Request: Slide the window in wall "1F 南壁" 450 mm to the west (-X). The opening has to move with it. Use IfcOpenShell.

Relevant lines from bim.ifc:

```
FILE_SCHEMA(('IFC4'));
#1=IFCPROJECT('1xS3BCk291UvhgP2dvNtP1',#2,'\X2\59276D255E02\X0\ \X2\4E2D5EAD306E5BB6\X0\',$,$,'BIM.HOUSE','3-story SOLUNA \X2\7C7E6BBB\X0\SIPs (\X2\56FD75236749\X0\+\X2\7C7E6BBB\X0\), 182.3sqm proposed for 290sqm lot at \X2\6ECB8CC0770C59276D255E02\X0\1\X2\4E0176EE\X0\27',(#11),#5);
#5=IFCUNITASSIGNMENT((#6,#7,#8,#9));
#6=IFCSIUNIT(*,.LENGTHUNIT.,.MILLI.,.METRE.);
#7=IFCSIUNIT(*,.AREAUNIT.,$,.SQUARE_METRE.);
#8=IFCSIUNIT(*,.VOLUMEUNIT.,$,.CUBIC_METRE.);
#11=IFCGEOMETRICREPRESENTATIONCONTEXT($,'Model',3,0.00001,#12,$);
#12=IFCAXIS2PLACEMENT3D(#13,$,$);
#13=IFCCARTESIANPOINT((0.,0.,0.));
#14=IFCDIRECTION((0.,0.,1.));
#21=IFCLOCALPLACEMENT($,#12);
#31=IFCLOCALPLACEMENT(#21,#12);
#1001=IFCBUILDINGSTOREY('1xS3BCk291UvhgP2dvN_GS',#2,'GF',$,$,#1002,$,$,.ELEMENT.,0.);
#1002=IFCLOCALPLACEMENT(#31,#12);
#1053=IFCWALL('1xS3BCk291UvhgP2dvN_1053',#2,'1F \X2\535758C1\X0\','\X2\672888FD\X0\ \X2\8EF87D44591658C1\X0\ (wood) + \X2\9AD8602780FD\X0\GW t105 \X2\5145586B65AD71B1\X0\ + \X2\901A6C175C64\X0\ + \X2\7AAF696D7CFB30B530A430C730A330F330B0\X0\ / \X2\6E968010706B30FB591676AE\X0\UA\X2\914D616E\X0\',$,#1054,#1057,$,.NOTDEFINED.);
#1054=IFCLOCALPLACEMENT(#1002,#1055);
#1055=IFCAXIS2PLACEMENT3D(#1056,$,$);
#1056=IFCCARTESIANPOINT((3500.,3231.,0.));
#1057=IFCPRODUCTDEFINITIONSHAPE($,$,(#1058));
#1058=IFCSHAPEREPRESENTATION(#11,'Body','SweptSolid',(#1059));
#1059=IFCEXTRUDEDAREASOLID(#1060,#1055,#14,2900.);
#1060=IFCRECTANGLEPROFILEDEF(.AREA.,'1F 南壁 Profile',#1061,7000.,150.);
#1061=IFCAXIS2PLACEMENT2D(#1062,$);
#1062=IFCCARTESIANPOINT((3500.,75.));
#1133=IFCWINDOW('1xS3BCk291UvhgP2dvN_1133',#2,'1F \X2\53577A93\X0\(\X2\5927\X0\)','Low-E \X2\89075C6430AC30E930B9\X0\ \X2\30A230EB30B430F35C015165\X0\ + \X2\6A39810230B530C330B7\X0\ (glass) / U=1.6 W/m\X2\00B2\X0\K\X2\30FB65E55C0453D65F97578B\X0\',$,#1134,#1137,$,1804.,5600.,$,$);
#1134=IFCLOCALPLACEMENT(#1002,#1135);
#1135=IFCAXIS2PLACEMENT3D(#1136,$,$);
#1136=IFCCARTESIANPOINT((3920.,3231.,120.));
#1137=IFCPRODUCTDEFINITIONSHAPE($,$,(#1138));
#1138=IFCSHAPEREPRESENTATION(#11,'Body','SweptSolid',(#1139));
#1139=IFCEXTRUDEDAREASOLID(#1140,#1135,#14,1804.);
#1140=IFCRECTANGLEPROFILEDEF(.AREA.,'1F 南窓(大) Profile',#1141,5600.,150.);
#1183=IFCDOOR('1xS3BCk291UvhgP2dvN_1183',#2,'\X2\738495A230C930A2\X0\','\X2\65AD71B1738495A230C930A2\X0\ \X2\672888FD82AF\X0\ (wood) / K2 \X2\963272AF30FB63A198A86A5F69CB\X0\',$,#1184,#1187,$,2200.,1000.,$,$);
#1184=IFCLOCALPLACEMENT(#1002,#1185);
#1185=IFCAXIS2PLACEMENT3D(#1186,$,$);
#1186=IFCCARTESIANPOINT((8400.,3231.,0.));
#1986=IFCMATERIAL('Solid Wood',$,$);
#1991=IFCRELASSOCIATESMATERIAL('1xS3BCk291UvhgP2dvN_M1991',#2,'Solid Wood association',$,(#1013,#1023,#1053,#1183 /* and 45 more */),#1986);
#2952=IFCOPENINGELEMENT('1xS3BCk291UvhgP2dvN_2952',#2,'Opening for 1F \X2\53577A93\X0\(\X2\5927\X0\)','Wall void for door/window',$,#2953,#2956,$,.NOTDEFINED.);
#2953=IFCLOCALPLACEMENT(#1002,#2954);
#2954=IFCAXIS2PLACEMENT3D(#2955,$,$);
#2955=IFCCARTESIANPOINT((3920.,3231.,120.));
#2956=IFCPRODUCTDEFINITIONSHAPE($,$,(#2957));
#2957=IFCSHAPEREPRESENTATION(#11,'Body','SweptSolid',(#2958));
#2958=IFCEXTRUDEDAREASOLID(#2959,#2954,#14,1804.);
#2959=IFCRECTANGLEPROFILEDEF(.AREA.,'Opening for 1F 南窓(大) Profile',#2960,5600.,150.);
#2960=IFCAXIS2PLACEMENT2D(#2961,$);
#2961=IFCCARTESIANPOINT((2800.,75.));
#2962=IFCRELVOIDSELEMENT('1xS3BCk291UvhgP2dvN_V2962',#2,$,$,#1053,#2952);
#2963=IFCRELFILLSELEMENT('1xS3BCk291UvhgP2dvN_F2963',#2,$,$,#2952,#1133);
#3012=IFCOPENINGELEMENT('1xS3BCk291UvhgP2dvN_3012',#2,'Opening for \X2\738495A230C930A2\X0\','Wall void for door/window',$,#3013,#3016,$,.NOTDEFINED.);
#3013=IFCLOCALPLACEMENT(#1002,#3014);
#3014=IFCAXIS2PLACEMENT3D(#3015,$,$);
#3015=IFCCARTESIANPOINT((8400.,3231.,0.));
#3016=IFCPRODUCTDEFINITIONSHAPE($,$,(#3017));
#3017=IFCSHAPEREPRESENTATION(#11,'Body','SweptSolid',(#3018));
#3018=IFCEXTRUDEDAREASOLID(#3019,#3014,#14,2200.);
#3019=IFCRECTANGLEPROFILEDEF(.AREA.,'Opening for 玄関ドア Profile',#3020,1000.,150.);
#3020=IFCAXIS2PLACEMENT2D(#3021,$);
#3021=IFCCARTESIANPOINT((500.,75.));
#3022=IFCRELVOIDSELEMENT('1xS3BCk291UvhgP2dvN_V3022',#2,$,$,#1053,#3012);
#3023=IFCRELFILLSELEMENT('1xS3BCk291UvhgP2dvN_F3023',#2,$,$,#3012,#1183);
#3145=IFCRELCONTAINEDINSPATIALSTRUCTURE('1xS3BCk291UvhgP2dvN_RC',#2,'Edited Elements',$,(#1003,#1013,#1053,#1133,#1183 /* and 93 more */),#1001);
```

```python
import ifcopenshell
import ifcopenshell.api.geometry
import ifcopenshell.util.placement

model = ifcopenshell.open("bim.ifc")

window = model.by_guid("1xS3BCk291UvhgP2dvN_1133")
opening = window.FillsVoids[0].RelatingOpeningElement
wall = opening.VoidsElements[0].RelatingBuildingElement

wall_matrix = ifcopenshell.util.placement.get_local_placement(wall.ObjectPlacement)
shift = wall_matrix[:3, 0] * -450.0
before = ifcopenshell.util.placement.get_local_placement(window.ObjectPlacement)[:3, 3].copy()

# The window is not placed relative to its opening, so move both.
for product in (opening, window):
    matrix = ifcopenshell.util.placement.get_local_placement(product.ObjectPlacement)
    matrix[:3, 3] += shift
    ifcopenshell.api.geometry.edit_object_placement(model, product=product, matrix=matrix, is_si=False)

after = ifcopenshell.util.placement.get_local_placement(window.ObjectPlacement)[:3, 3]
print("window moved by", (after - before).round(3) + 0.0)

model.write("bim-out.ifc")
```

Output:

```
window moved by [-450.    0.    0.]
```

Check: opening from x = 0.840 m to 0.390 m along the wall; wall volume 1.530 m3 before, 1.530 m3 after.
